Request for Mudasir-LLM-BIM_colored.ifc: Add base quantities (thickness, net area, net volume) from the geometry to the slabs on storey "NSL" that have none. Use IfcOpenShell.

First a look at what the model holds.

```python
import ifcopenshell
import ifcopenshell.util.element
import ifcopenshell.util.unit

model = ifcopenshell.open("Mudasir-LLM-BIM_colored.ifc")
print(model.schema)
for unit_type in ("LENGTHUNIT", "AREAUNIT", "VOLUMEUNIT"):
    print(unit_type, ifcopenshell.util.unit.calculate_unit_scale(model, unit_type))
storey = next(s for s in model.by_type("IfcBuildingStorey") if s.Name == "NSL")
slabs = [e for e in ifcopenshell.util.element.get_decomposition(storey) if e.is_a("IfcSlab")]
for e in sorted(slabs, key=lambda e: e.id()):
    print(e.id(), e.is_a(), e.Name, list(ifcopenshell.util.element.get_psets(e, qtos_only=True)), sep=" | ")
```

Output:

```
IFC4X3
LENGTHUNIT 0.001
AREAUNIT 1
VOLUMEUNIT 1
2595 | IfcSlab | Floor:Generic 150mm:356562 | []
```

```python
import ifcopenshell
import ifcopenshell.api.pset
import ifcopenshell.geom
import ifcopenshell.util.element
import ifcopenshell.util.shape
import ifcopenshell.util.unit

model = ifcopenshell.open("Mudasir-LLM-BIM_colored.ifc")
unit_scale = ifcopenshell.util.unit.calculate_unit_scale(model)
area_scale = ifcopenshell.util.unit.calculate_unit_scale(model, "AREAUNIT")
volume_scale = ifcopenshell.util.unit.calculate_unit_scale(model, "VOLUMEUNIT")
settings = ifcopenshell.geom.settings()

storey = next(s for s in model.by_type("IfcBuildingStorey") if s.Name == "NSL")
slabs = [e for e in ifcopenshell.util.element.get_decomposition(storey) if e.is_a("IfcSlab")]

for e in sorted(slabs, key=lambda e: e.id()):
    if ifcopenshell.util.element.get_psets(e, qtos_only=True, should_inherit=False):
        continue
    # Geometry comes back in metres, in the element's own axes.
    shape = ifcopenshell.geom.create_shape(settings, e)
    values = {
        "Width": ifcopenshell.util.shape.get_z(shape.geometry) / unit_scale,
        "NetArea": ifcopenshell.util.shape.get_footprint_area(shape.geometry) / area_scale,
        "NetVolume": ifcopenshell.util.shape.get_volume(shape.geometry) / volume_scale,
    }
    qto = ifcopenshell.api.pset.add_qto(model, product=e, name="Qto_SlabBaseQuantities")
    ifcopenshell.api.pset.edit_qto(model, qto=qto, properties=values)
    print(e.id(), {k: round(v, 3) for k, v in values.items()})

model.write("Mudasir-LLM-BIM_colored_edited.ifc")
```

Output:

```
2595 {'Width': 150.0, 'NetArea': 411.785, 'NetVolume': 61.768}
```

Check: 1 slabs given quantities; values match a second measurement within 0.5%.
